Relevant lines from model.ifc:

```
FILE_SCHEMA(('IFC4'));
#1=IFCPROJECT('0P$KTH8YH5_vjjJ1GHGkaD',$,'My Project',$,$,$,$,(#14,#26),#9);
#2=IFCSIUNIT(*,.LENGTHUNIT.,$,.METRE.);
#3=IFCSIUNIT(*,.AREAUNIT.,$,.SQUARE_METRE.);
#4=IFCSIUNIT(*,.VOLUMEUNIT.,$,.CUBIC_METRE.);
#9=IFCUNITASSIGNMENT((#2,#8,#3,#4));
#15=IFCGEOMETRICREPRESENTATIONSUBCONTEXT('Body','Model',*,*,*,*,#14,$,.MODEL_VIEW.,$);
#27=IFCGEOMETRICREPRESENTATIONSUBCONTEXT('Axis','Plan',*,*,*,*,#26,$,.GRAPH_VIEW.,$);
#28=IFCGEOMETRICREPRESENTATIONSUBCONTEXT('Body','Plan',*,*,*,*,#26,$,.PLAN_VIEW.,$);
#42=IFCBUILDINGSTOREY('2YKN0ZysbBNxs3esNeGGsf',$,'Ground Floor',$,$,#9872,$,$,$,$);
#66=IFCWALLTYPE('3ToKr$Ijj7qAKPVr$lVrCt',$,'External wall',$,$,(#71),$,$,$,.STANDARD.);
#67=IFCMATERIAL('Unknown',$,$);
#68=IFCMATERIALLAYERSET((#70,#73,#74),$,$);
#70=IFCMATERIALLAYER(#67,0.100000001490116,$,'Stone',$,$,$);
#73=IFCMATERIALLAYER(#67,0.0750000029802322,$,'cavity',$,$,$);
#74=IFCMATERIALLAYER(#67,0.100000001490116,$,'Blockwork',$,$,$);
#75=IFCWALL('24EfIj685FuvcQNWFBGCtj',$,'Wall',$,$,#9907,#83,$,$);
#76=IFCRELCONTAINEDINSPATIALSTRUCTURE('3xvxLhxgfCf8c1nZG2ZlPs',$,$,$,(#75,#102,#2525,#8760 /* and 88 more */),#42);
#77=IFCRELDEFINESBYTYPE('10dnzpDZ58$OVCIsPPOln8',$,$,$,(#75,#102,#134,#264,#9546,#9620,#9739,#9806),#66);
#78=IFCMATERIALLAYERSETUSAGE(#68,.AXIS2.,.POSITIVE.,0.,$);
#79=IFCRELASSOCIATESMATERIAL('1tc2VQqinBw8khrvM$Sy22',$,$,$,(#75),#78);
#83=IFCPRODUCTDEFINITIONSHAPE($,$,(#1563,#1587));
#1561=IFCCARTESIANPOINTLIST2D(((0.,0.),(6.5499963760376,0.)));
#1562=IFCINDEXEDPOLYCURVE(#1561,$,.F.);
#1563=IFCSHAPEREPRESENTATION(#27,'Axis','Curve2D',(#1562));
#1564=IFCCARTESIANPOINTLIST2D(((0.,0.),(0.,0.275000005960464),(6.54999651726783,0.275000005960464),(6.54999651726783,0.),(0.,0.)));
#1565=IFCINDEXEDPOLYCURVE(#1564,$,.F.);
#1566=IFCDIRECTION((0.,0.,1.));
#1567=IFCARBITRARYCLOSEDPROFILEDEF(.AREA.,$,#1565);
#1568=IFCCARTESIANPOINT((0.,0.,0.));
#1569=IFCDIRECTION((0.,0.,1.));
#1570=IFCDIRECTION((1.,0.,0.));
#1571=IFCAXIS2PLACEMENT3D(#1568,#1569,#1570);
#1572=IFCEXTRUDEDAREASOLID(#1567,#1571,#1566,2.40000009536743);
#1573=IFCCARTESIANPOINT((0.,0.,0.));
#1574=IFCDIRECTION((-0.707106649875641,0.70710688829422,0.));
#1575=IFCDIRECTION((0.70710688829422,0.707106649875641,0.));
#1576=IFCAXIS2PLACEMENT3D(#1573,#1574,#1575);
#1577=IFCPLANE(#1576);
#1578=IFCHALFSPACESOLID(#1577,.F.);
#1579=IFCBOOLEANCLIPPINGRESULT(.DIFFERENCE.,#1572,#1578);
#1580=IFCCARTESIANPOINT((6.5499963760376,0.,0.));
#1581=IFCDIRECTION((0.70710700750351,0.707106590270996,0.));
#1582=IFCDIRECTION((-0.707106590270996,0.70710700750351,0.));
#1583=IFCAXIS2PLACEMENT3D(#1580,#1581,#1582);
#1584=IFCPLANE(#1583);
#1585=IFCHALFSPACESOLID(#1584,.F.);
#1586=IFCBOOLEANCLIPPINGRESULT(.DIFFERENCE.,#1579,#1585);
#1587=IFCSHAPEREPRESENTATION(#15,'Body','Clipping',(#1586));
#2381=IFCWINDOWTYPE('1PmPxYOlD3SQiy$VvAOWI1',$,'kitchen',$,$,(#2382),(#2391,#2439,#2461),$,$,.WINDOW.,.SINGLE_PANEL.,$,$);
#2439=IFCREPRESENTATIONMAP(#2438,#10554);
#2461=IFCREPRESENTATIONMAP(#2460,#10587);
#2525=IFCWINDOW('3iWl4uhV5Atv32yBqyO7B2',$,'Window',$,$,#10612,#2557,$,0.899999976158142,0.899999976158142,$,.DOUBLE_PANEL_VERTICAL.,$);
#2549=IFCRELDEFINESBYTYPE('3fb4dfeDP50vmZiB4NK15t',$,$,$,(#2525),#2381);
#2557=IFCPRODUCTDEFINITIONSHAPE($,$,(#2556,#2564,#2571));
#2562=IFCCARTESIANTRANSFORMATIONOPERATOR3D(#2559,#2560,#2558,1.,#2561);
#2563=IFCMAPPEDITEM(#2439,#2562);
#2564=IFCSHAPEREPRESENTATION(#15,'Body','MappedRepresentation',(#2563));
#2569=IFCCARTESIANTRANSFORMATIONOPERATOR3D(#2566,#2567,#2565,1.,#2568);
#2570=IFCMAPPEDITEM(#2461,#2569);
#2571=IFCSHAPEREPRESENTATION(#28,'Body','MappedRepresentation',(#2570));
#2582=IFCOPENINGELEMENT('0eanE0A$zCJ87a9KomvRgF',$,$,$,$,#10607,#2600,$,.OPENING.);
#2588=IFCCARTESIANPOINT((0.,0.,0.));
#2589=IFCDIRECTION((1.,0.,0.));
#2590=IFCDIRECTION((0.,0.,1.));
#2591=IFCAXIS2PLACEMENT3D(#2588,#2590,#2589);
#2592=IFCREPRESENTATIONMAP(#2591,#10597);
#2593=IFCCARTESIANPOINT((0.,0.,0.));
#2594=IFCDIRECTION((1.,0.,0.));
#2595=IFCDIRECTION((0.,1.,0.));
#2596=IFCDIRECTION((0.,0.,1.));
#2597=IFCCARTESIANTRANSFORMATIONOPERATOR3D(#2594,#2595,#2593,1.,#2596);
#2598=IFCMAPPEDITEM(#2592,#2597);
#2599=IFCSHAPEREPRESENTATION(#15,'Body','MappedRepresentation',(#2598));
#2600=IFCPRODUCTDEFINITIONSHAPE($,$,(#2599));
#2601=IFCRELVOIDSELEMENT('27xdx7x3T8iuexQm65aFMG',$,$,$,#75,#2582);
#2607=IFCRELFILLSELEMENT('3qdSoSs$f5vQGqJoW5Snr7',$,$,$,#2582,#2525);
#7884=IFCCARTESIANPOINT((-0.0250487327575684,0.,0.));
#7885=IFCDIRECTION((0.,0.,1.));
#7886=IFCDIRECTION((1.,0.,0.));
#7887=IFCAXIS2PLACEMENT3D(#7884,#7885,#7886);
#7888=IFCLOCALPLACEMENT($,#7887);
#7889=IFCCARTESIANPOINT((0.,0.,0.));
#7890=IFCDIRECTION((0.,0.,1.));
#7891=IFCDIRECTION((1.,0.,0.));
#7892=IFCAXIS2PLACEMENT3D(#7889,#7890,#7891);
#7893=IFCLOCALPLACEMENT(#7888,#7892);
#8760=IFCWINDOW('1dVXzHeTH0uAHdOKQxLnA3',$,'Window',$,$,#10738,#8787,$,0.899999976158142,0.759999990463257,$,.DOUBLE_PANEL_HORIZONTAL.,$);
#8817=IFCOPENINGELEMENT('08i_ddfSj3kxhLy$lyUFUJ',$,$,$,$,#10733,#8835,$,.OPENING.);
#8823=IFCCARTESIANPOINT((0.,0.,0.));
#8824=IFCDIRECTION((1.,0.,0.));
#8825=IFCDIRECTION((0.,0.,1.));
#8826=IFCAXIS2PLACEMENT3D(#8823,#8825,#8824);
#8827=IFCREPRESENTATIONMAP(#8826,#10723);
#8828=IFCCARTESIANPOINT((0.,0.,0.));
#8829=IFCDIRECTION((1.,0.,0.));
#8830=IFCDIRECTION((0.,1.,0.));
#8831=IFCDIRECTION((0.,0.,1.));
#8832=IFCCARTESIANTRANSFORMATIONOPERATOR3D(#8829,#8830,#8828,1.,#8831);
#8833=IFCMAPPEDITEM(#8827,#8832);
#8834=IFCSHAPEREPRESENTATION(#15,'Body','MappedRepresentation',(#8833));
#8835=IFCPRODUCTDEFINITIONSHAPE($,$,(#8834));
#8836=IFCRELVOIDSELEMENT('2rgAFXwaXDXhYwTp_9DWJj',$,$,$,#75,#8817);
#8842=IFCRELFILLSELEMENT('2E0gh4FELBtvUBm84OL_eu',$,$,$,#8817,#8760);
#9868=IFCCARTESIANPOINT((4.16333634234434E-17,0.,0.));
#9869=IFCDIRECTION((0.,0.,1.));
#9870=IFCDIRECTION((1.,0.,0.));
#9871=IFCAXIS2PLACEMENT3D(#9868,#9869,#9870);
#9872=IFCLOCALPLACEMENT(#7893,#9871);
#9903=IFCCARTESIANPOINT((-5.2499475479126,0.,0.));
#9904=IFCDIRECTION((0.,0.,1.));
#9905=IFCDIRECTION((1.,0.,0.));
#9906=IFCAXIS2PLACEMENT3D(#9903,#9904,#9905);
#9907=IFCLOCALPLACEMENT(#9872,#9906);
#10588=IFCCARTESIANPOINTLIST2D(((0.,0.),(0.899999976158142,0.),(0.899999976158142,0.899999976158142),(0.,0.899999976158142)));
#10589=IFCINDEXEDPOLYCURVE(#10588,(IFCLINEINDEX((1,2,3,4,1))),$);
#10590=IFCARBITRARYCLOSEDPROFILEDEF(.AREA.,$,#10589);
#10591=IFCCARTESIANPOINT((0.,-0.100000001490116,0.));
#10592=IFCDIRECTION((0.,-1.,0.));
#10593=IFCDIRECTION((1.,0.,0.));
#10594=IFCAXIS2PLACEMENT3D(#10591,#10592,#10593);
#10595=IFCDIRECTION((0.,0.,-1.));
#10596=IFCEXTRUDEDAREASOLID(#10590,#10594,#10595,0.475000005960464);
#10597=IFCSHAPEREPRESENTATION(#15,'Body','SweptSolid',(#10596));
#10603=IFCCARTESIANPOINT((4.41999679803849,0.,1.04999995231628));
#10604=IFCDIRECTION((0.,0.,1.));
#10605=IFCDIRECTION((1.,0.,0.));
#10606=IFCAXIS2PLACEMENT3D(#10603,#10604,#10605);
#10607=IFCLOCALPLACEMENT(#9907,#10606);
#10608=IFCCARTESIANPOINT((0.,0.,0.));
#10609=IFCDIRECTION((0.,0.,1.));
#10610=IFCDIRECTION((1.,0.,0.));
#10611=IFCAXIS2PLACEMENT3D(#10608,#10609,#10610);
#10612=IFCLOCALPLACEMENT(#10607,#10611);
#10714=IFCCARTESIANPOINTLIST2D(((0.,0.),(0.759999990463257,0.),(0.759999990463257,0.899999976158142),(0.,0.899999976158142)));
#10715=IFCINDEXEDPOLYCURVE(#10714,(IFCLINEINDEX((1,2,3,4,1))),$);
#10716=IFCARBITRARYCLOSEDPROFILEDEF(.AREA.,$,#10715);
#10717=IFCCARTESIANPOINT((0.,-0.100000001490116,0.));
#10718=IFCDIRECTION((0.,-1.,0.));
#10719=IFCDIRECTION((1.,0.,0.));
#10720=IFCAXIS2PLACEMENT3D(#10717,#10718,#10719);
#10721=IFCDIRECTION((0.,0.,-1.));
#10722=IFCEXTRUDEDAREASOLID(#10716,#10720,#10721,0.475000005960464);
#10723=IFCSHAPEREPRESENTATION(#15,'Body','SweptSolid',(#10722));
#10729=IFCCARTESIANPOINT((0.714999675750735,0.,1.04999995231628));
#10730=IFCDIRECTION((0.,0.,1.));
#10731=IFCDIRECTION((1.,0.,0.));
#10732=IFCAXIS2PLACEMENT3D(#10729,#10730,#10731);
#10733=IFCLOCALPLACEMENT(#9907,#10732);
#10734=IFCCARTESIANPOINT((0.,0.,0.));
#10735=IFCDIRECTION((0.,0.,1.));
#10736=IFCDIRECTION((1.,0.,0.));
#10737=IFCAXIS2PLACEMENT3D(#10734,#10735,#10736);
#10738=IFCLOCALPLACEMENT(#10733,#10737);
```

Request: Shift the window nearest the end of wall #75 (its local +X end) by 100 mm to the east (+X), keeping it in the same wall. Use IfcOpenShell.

```python
import ifcopenshell
import ifcopenshell.api.geometry
import ifcopenshell.util.placement

model = ifcopenshell.open("model.ifc")

window = model.by_guid("3iWl4uhV5Atv32yBqyO7B2")
opening = window.FillsVoids[0].RelatingOpeningElement
wall = opening.VoidsElements[0].RelatingBuildingElement

wall_matrix = ifcopenshell.util.placement.get_local_placement(wall.ObjectPlacement)
shift = wall_matrix[:3, 0] * 0.1
before = ifcopenshell.util.placement.get_local_placement(window.ObjectPlacement)[:3, 3].copy()

# The window is placed relative to its opening, so it follows when the opening moves.
matrix = ifcopenshell.util.placement.get_local_placement(opening.ObjectPlacement)
matrix[:3, 3] += shift
ifcopenshell.api.geometry.edit_object_placement(
    model, product=opening, matrix=matrix, is_si=False, should_transform_children=True
)

after = ifcopenshell.util.placement.get_local_placement(window.ObjectPlacement)[:3, 3]
print("window moved by", (after - before).round(3) + 0.0)

model.write("model_edited.ifc")
```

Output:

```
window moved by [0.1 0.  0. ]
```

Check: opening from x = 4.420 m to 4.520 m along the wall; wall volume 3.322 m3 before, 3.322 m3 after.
